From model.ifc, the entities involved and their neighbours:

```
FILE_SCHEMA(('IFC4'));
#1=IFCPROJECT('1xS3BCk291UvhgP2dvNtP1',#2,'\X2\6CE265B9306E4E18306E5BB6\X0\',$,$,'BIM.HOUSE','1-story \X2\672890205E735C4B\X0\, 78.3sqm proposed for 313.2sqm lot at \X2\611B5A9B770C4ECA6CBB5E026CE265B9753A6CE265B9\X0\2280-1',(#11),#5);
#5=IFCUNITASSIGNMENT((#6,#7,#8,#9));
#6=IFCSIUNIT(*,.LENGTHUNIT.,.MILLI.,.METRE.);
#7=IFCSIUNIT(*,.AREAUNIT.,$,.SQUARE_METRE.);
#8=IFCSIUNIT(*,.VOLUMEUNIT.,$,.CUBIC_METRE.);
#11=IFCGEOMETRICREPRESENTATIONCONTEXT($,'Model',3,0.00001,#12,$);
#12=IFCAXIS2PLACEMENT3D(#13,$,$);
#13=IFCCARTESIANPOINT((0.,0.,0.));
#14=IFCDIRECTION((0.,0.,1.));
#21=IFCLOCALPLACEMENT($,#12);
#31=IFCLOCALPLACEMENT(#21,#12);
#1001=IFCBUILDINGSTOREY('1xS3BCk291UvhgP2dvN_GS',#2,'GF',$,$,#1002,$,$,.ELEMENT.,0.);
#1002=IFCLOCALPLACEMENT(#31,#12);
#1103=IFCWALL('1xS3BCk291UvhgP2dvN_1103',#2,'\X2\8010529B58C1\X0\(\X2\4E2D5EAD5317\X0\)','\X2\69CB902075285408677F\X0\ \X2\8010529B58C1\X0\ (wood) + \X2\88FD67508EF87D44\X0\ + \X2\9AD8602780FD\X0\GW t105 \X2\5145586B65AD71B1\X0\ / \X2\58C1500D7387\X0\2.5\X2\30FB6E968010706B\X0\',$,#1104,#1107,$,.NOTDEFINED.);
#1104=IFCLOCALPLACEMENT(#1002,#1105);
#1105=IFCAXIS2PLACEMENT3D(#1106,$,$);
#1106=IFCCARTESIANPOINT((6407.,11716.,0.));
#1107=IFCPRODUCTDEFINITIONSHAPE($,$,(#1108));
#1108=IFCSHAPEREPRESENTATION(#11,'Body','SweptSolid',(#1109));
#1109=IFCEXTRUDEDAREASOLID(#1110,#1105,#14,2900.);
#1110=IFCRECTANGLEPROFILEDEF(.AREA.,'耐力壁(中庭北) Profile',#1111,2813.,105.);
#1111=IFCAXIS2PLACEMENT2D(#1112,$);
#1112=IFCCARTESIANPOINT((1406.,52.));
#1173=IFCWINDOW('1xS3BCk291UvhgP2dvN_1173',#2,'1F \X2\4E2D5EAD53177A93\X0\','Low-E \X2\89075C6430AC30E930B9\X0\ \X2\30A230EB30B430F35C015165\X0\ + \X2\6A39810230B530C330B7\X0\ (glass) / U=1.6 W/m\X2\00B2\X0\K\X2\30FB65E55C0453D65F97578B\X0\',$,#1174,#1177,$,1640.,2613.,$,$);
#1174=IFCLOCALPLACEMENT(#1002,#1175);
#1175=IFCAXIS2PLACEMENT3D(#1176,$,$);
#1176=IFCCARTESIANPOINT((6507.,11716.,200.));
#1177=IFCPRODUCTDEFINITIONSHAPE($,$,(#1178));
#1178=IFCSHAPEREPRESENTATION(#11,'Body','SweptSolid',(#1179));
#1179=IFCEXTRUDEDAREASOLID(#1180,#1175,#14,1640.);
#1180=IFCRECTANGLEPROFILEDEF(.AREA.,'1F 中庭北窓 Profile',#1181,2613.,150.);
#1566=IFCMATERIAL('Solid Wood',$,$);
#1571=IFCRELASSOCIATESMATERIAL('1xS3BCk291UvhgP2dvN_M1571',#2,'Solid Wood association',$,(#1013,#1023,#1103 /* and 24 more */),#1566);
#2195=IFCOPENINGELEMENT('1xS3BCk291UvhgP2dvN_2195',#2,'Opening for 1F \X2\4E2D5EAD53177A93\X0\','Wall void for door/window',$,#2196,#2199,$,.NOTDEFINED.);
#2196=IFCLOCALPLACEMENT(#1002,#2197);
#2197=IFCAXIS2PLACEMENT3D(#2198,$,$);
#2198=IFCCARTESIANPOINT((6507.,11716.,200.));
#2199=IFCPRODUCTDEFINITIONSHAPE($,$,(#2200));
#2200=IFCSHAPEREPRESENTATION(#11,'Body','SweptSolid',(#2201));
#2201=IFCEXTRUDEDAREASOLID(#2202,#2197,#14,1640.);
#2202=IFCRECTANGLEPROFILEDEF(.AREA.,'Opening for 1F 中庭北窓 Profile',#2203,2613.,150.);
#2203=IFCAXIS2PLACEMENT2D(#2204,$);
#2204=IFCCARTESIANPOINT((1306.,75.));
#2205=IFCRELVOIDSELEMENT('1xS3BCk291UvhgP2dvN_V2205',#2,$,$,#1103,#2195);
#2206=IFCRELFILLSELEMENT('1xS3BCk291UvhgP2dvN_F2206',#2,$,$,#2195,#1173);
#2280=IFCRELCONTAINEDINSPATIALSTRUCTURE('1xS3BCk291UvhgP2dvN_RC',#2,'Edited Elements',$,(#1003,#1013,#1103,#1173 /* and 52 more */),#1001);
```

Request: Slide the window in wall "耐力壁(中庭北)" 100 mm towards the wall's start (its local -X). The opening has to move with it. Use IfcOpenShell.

```python
import ifcopenshell
import ifcopenshell.api.geometry
import ifcopenshell.util.placement

model = ifcopenshell.open("model.ifc")

window = model.by_id(1173)
opening = window.FillsVoids[0].RelatingOpeningElement
wall = opening.VoidsElements[0].RelatingBuildingElement

wall_matrix = ifcopenshell.util.placement.get_local_placement(wall.ObjectPlacement)
shift = wall_matrix[:3, 0] * -100.0
before = ifcopenshell.util.placement.get_local_placement(window.ObjectPlacement)[:3, 3].copy()

# The window is not placed relative to its opening, so move both.
for product in (opening, window):
    matrix = ifcopenshell.util.placement.get_local_placement(product.ObjectPlacement)
    matrix[:3, 3] += shift
    ifcopenshell.api.geometry.edit_object_placement(model, product=product, matrix=matrix, is_si=False)

after = ifcopenshell.util.placement.get_local_placement(window.ObjectPlacement)[:3, 3]
print("window moved by", (after - before).round(3) + 0.0)

model.write("model-out.ifc")
```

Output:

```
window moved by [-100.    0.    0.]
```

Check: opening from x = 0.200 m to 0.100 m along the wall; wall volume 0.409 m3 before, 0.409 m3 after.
